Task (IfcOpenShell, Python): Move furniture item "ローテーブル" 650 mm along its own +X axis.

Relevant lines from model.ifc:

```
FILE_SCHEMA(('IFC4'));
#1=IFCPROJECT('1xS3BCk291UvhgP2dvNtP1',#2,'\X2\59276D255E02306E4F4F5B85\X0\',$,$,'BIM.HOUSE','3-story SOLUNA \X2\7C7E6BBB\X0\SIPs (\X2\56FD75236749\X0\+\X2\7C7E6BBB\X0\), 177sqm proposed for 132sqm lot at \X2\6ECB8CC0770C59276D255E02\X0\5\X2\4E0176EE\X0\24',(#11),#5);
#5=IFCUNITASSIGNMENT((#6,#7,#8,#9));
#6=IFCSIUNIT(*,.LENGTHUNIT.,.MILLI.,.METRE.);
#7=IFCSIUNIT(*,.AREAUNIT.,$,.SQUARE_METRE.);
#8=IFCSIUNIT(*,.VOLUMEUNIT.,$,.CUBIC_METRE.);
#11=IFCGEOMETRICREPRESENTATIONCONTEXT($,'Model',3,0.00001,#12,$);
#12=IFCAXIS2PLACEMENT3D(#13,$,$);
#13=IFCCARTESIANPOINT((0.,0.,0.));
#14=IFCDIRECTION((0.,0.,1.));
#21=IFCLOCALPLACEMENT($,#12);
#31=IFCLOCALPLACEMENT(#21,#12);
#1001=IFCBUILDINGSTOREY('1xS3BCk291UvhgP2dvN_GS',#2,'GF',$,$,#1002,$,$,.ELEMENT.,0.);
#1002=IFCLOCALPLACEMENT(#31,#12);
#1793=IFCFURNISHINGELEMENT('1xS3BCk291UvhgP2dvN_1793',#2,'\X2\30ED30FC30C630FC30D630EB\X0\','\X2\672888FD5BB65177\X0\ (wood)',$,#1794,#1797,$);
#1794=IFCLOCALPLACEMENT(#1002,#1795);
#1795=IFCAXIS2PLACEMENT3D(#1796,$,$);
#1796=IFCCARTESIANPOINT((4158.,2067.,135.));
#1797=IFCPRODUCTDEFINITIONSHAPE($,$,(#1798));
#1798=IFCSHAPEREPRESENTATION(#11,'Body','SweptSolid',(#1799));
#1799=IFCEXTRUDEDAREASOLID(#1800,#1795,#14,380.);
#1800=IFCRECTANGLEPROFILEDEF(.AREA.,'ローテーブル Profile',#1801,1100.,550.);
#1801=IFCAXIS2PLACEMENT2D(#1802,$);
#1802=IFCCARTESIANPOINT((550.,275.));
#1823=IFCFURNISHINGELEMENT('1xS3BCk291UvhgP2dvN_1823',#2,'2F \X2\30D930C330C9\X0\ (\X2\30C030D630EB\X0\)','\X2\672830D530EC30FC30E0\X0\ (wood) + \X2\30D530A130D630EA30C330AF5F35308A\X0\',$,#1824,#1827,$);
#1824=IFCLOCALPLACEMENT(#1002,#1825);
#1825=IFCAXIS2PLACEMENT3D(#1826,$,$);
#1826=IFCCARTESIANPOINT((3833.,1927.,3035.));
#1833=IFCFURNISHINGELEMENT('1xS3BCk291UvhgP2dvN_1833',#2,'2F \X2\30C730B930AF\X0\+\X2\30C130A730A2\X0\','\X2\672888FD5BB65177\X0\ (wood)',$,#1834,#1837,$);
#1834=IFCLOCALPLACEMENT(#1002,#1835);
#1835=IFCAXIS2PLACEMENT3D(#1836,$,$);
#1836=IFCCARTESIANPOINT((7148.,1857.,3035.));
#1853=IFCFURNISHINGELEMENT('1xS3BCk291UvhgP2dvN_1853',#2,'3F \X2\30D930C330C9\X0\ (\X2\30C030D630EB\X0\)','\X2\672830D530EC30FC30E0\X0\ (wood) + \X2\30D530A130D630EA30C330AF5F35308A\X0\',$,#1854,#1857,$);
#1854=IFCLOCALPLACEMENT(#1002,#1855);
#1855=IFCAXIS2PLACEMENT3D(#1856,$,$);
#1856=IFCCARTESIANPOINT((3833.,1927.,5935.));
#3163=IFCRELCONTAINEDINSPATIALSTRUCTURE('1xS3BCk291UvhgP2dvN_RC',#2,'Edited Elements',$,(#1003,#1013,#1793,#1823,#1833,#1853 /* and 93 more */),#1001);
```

```python
import ifcopenshell
import ifcopenshell.api.geometry
import ifcopenshell.util.placement

model = ifcopenshell.open("model.ifc")

item = model.by_id(1793)
matrix = ifcopenshell.util.placement.get_local_placement(item.ObjectPlacement)
matrix[:3, 3] += matrix[:3, 0] * 650.0
ifcopenshell.api.geometry.edit_object_placement(model, product=item, matrix=matrix, is_si=False)

print(ifcopenshell.util.placement.get_local_placement(item.ObjectPlacement).round(3) + 0.0)

model.write("model_rev.ifc")
```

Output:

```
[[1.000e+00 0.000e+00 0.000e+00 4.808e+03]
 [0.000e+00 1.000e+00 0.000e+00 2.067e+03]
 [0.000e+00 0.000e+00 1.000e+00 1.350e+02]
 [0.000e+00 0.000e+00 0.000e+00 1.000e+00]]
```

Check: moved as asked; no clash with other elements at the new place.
